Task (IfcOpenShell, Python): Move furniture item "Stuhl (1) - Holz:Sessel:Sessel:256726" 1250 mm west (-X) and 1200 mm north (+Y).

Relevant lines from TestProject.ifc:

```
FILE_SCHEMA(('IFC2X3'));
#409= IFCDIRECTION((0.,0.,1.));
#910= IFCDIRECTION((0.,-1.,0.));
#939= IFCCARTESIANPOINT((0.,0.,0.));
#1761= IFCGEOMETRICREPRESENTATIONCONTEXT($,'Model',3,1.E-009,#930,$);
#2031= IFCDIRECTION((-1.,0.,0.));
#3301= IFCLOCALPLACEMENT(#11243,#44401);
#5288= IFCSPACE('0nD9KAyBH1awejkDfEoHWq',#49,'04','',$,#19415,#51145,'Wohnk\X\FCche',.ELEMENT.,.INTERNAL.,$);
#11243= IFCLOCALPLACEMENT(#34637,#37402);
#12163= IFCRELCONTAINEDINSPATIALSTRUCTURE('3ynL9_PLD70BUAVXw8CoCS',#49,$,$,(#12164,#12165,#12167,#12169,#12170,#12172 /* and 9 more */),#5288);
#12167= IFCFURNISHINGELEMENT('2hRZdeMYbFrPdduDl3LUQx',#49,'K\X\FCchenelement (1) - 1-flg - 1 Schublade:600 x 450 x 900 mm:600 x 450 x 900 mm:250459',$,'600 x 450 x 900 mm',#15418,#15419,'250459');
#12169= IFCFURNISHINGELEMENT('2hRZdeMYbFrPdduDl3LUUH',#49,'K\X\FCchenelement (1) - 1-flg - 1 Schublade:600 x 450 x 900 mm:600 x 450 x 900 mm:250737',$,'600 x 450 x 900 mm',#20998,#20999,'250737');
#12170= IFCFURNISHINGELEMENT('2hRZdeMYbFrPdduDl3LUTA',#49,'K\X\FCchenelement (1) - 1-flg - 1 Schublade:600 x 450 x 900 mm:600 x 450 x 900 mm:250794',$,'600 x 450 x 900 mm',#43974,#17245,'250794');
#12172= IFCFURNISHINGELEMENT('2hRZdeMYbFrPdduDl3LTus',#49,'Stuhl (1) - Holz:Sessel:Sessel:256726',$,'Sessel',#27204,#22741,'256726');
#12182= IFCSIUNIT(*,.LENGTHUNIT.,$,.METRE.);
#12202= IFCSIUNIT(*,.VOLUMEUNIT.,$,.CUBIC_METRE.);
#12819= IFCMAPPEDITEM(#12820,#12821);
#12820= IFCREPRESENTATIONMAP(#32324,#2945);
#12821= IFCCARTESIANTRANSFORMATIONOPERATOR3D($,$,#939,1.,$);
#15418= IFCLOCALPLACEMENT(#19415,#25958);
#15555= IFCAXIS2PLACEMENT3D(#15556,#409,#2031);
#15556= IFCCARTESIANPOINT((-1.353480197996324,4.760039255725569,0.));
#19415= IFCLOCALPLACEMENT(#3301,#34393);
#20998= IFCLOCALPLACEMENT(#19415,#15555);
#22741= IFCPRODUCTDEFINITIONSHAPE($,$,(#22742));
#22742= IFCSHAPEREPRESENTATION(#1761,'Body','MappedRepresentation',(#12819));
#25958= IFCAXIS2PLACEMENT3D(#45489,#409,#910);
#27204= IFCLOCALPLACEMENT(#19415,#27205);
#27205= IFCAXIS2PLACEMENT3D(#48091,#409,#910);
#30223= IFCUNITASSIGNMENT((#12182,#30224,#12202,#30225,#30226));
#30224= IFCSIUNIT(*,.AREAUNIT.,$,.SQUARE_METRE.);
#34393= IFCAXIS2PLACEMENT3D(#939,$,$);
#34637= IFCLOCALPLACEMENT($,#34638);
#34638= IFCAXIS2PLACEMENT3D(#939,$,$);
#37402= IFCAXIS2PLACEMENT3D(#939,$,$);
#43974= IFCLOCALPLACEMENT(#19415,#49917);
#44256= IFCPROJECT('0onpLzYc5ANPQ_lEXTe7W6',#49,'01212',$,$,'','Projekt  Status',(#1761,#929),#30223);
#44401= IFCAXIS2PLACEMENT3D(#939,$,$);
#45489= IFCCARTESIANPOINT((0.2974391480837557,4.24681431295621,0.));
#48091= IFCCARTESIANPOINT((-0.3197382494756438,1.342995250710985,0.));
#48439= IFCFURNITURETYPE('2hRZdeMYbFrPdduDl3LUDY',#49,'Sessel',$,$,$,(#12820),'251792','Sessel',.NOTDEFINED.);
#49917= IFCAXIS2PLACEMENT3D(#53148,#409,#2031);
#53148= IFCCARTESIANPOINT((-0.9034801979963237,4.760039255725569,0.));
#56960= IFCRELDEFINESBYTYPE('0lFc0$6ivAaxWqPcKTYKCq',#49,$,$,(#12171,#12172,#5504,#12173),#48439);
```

```python
import ifcopenshell
import ifcopenshell.api.geometry
import ifcopenshell.util.placement
import ifcopenshell.util.unit

model = ifcopenshell.open("TestProject.ifc")
unit_scale = ifcopenshell.util.unit.calculate_unit_scale(model)

item = model.by_guid("2hRZdeMYbFrPdduDl3LTus")
matrix = ifcopenshell.util.placement.get_local_placement(item.ObjectPlacement)
matrix[0, 3] -= 1.25 / unit_scale
matrix[1, 3] += 1.2 / unit_scale
ifcopenshell.api.geometry.edit_object_placement(model, product=item, matrix=matrix, is_si=False)

print(ifcopenshell.util.placement.get_local_placement(item.ObjectPlacement).round(3) + 0.0)

model.write("TestProject-out.ifc")
```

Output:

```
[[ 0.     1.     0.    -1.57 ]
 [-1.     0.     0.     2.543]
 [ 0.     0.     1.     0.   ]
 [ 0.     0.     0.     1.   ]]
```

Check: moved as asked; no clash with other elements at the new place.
